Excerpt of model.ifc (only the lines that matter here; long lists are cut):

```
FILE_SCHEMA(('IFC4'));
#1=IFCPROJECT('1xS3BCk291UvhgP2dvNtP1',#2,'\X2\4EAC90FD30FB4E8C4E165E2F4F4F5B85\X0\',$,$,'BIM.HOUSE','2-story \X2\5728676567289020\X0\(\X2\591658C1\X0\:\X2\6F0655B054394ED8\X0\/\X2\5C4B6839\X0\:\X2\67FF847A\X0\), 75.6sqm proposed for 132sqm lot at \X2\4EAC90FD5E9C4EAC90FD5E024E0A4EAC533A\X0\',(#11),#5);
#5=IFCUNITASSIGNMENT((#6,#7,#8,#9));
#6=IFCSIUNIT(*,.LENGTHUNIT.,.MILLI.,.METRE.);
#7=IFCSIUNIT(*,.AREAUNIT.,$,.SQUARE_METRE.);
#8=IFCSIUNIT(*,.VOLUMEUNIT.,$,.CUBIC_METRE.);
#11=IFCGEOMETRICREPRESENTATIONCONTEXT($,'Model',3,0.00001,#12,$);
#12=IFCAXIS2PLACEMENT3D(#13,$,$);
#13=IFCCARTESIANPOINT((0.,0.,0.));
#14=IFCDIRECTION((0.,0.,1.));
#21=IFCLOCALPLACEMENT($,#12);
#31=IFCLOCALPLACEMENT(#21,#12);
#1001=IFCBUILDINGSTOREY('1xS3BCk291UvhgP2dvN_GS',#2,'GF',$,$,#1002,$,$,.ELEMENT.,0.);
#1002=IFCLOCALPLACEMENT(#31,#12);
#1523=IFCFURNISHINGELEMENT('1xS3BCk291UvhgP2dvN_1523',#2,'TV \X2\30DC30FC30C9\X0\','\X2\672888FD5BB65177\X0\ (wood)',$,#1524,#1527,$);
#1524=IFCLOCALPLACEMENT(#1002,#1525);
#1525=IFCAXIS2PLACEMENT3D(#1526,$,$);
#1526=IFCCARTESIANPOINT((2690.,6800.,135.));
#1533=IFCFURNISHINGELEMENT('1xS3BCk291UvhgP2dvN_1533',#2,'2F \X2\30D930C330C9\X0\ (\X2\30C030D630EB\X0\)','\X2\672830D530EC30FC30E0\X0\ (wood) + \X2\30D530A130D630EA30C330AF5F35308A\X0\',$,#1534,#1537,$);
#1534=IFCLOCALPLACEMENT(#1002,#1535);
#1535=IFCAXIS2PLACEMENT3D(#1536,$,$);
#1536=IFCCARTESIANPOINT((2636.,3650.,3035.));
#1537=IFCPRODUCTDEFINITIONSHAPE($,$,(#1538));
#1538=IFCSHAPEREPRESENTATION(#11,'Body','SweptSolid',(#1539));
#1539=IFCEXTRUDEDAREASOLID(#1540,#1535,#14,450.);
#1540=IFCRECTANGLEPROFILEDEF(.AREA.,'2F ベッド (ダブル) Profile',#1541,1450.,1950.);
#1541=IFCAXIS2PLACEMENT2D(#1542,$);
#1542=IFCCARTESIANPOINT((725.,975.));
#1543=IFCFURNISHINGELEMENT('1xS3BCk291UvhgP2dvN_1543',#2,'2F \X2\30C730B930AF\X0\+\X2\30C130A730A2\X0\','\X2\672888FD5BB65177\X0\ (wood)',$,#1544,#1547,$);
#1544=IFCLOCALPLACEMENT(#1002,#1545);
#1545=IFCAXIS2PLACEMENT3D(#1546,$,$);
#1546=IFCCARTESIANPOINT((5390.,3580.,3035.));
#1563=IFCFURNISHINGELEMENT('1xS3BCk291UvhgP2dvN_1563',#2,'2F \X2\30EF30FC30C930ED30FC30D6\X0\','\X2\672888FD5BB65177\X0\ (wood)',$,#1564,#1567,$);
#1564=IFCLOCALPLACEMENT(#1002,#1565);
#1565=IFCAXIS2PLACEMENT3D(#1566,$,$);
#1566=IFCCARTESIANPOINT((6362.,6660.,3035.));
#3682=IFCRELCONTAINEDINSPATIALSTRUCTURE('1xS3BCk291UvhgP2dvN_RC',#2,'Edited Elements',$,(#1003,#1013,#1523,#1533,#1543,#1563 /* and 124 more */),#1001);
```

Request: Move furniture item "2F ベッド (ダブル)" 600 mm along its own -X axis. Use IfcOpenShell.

```python
import ifcopenshell
import ifcopenshell.api.geometry
import ifcopenshell.util.placement
import ifcopenshell.util.unit

model = ifcopenshell.open("model.ifc")
unit_scale = ifcopenshell.util.unit.calculate_unit_scale(model)

item = model.by_guid("1xS3BCk291UvhgP2dvN_1533")
matrix = ifcopenshell.util.placement.get_local_placement(item.ObjectPlacement)
matrix[:3, 3] -= matrix[:3, 0] * 0.6 / unit_scale
ifcopenshell.api.geometry.edit_object_placement(model, product=item, matrix=matrix, is_si=False)

print(ifcopenshell.util.placement.get_local_placement(item.ObjectPlacement).round(3) + 0.0)

model.write("model_updated.ifc")
```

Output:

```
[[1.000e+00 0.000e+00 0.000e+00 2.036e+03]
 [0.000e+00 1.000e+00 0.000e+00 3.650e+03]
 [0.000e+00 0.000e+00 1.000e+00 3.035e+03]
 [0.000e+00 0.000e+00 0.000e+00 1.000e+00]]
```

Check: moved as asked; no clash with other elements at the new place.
